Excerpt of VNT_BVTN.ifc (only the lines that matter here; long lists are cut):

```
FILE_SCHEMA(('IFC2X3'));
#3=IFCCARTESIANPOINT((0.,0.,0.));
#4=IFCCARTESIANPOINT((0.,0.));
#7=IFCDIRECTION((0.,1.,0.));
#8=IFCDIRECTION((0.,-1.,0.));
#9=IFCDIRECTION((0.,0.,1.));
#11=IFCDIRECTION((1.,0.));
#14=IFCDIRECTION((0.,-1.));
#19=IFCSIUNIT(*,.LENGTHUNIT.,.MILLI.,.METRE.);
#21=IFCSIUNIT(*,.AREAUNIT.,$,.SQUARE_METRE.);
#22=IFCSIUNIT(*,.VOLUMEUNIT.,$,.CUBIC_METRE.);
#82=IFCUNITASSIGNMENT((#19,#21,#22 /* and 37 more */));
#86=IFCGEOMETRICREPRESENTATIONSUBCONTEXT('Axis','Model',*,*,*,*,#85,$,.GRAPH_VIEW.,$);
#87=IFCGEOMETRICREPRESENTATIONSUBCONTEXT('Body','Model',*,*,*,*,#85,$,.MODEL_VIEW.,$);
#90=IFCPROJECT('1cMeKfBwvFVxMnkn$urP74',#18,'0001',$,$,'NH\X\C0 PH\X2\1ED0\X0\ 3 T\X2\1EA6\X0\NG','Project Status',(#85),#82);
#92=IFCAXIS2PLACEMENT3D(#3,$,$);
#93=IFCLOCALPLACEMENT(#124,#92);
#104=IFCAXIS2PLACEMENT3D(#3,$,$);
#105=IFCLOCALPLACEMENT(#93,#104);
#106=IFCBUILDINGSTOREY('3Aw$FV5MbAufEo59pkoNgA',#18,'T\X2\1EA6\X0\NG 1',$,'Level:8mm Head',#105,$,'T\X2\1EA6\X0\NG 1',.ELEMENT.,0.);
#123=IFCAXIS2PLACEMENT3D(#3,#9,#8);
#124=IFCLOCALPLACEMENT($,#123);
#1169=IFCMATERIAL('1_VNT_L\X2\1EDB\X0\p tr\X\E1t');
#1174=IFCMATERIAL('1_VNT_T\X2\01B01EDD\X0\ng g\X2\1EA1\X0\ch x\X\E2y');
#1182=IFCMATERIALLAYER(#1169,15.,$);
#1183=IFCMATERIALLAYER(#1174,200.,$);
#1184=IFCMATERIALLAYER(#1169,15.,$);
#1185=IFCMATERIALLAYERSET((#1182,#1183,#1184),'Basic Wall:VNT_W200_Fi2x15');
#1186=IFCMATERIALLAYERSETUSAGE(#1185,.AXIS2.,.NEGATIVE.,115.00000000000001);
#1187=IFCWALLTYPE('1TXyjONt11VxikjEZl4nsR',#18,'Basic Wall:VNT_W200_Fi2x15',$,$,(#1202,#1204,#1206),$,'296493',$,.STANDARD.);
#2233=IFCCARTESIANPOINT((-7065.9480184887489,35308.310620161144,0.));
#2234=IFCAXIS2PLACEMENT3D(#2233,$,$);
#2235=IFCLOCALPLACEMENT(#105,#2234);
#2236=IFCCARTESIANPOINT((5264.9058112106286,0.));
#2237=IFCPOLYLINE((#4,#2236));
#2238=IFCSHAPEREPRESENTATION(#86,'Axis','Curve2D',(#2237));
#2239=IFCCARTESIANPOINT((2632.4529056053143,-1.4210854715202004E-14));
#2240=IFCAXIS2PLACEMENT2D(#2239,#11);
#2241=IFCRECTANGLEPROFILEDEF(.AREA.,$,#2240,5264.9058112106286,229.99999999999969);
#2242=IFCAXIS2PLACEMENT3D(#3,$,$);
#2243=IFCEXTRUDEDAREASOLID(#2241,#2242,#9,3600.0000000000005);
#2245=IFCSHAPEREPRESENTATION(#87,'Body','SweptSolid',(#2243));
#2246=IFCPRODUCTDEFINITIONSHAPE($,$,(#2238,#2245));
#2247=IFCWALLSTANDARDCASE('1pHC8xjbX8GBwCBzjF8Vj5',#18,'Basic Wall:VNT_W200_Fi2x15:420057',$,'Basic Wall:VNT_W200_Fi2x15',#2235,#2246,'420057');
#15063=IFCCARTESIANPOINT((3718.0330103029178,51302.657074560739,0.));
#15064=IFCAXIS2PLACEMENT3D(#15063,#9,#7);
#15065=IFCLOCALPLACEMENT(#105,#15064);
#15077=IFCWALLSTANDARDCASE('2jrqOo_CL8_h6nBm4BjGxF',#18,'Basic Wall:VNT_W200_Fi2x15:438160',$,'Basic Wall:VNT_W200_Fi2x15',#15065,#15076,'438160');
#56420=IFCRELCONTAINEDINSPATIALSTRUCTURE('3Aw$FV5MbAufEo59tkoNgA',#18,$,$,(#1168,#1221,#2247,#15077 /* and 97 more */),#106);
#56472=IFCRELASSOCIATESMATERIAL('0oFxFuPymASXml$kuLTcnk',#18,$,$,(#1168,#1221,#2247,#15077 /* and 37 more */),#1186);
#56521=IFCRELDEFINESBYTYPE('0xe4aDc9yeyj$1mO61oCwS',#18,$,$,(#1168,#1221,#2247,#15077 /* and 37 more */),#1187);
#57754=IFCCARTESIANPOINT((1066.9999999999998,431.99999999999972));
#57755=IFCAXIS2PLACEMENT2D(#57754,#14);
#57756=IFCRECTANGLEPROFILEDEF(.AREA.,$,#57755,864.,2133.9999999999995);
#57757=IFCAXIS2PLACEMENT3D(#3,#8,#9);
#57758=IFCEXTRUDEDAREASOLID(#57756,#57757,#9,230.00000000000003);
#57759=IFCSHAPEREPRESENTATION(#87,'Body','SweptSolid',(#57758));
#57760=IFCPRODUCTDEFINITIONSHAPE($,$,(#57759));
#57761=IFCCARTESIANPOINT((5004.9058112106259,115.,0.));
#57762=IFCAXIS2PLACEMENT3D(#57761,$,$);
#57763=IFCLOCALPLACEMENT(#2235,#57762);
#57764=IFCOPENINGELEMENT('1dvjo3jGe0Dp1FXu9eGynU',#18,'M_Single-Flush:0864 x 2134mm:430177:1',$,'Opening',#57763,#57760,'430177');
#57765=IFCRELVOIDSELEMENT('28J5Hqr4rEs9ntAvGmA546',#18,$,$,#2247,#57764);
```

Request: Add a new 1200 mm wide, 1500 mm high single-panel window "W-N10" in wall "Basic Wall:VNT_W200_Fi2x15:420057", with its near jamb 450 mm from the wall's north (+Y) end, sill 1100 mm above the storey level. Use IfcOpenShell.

```python
import numpy as np
import ifcopenshell
import ifcopenshell.api.feature
import ifcopenshell.api.geometry
import ifcopenshell.api.root
import ifcopenshell.api.spatial
import ifcopenshell.api.type
import ifcopenshell.geom
import ifcopenshell.util.element
import ifcopenshell.util.placement
import ifcopenshell.util.representation
import ifcopenshell.util.shape
import ifcopenshell.util.unit

model = ifcopenshell.open("VNT_BVTN.ifc")
unit_scale = ifcopenshell.util.unit.calculate_unit_scale(model)
settings = ifcopenshell.geom.settings()


def volume(element):
    """Net volume in cubic metres, openings subtracted."""
    shape = ifcopenshell.geom.create_shape(settings, element)
    return ifcopenshell.util.shape.get_volume(shape.geometry)


wall = model.by_guid("1pHC8xjbX8GBwCBzjF8Vj5")
storey = ifcopenshell.util.element.get_container(wall, ifc_class="IfcBuildingStorey")
context = ifcopenshell.util.representation.get_context(model, "Model", "Body", "MODEL_VIEW")
before = volume(wall)

width, height, from_end, sill = 1.2, 1.5, 0.45, 1.1  # metres

# The wall runs along its own X axis, and the end named is its -X end.
wall_shape = ifcopenshell.geom.create_shape(settings, wall)
x, y, z = ifcopenshell.util.shape.get_vertices(wall_shape.geometry).T
start = x.min() + from_end
face, thickness = float(y.min()), float(y.max() - y.min())
wall_matrix = ifcopenshell.util.placement.get_local_placement(wall.ObjectPlacement)
level = ifcopenshell.util.placement.get_local_placement(storey.ObjectPlacement)[2, 3]


def in_wall(x, y):
    """Placement at x, y metres in the wall's axes, at sill height."""
    matrix = wall_matrix.copy()
    matrix[:, 3] = wall_matrix @ np.array([x / unit_scale, y / unit_scale, 0.0, 1.0])
    matrix[2, 3] = level + sill / unit_scale
    return matrix


# Opening: a box that overshoots both wall faces by 50 mm.
opening = ifcopenshell.api.root.create_entity(model, ifc_class="IfcOpeningElement")
box = ifcopenshell.api.geometry.add_wall_representation(
    model, context=context, length=width, height=height, thickness=thickness + 0.1
)
ifcopenshell.api.geometry.assign_representation(model, product=opening, representation=box)
ifcopenshell.api.geometry.edit_object_placement(model, product=opening, matrix=in_wall(start, face - 0.05), is_si=False)
ifcopenshell.api.feature.add_feature(model, feature=opening, element=wall)

window = ifcopenshell.api.root.create_entity(model, ifc_class="IfcWindow", name="W-N10")
window.OverallWidth, window.OverallHeight = width / unit_scale, height / unit_scale
body = ifcopenshell.api.geometry.add_window_representation(
    model,
    context=context,
    overall_width=window.OverallWidth,
    overall_height=window.OverallHeight,
    partition_type="SINGLE_PANEL",
)
ifcopenshell.api.geometry.assign_representation(model, product=window, representation=body)
ifcopenshell.api.spatial.assign_container(model, products=[window], relating_structure=storey)
fills = ifcopenshell.api.feature.add_filling(model, opening=opening, element=window)
fills.OwnerHistory = window.OwnerHistory  # required in IFC2X3

# IFC2X3 keeps the operation on the window style.
style = ifcopenshell.api.root.create_entity(model, ifc_class="IfcWindowStyle", name="W-N10")
style.OperationType, style.ConstructionType = "SINGLE_PANEL", "NOTDEFINED"
style.ParameterTakesPrecedence = style.Sizeable = False
ifcopenshell.api.type.assign_type(model, related_objects=[window], relating_type=style)

# Centre the window in the wall's thickness.
ifcopenshell.api.geometry.edit_object_placement(model, product=window, matrix=in_wall(start, face), is_si=False)
window_shape = ifcopenshell.geom.create_shape(settings, window)
depth = ifcopenshell.util.shape.get_vertices(window_shape.geometry)[:, 1]
offset = face + thickness / 2 - (depth.min() + depth.max()) / 2
ifcopenshell.api.geometry.edit_object_placement(model, product=window, matrix=in_wall(start, offset), is_si=False)

after = volume(wall)

print(f"wall volume {before:.3f} -> {after:.3f} m3")

model.write("VNT_BVTN-out.ifc")
```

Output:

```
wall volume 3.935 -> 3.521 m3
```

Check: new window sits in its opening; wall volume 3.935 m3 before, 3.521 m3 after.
